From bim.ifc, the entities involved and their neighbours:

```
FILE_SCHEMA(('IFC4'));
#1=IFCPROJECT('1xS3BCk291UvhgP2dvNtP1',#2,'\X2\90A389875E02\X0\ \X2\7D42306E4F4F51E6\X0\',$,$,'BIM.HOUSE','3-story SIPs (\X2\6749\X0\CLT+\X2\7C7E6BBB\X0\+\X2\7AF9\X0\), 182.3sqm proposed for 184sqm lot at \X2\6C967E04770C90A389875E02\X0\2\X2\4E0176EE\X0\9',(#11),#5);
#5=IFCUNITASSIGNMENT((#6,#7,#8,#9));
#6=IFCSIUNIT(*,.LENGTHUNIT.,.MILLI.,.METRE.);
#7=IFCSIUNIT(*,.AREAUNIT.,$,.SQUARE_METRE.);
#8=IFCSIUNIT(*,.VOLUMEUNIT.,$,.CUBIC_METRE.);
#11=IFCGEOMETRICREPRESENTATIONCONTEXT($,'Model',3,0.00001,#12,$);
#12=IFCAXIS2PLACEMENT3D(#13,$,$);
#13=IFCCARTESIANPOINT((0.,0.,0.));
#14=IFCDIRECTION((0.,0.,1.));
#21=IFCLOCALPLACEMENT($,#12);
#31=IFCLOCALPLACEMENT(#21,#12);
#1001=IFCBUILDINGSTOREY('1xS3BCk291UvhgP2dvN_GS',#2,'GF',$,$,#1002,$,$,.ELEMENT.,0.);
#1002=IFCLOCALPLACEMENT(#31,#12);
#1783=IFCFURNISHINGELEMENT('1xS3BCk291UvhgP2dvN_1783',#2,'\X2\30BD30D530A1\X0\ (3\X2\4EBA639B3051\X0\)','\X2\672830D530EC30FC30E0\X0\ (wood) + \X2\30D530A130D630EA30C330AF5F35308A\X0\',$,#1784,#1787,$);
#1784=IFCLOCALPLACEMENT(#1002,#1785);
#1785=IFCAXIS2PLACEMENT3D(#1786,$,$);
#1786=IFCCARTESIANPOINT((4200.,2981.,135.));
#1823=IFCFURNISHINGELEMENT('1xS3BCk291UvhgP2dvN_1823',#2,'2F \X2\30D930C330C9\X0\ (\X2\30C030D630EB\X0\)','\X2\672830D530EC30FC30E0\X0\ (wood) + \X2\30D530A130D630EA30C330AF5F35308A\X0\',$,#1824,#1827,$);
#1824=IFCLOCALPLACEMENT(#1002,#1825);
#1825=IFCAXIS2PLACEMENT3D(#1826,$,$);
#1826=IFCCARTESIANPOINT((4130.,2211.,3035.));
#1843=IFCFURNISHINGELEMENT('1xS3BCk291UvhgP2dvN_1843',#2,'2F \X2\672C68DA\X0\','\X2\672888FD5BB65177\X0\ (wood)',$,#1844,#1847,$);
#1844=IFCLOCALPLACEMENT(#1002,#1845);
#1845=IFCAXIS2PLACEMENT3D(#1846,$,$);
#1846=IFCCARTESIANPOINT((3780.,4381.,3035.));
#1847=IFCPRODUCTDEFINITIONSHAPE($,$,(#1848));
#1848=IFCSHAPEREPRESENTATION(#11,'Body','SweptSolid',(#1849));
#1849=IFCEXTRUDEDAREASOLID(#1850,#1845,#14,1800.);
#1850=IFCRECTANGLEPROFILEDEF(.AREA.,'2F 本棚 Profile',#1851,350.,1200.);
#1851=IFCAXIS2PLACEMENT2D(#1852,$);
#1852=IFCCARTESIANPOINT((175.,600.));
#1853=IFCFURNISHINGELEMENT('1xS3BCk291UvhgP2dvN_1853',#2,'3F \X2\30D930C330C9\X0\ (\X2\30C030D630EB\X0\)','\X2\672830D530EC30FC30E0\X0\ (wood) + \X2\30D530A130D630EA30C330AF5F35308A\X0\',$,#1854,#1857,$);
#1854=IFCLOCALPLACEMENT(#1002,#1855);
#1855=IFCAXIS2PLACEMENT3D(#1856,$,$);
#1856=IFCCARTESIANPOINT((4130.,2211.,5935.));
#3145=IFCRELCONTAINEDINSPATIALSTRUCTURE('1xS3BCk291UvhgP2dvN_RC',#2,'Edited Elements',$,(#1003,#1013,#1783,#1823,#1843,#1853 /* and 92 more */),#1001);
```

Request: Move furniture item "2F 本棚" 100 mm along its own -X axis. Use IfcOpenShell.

```python
import ifcopenshell
import ifcopenshell.api.geometry
import ifcopenshell.util.placement
import ifcopenshell.util.unit

model = ifcopenshell.open("bim.ifc")
unit_scale = ifcopenshell.util.unit.calculate_unit_scale(model)

item = model.by_guid("1xS3BCk291UvhgP2dvN_1843")
matrix = ifcopenshell.util.placement.get_local_placement(item.ObjectPlacement)
matrix[:3, 3] -= matrix[:3, 0] * 0.1 / unit_scale
ifcopenshell.api.geometry.edit_object_placement(model, product=item, matrix=matrix, is_si=False)

print(ifcopenshell.util.placement.get_local_placement(item.ObjectPlacement).round(3) + 0.0)

model.write("bim_updated.ifc")
```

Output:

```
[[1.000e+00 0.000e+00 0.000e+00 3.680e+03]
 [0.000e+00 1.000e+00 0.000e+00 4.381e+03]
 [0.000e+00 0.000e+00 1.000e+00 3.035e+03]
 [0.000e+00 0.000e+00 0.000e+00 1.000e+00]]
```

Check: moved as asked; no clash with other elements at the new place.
